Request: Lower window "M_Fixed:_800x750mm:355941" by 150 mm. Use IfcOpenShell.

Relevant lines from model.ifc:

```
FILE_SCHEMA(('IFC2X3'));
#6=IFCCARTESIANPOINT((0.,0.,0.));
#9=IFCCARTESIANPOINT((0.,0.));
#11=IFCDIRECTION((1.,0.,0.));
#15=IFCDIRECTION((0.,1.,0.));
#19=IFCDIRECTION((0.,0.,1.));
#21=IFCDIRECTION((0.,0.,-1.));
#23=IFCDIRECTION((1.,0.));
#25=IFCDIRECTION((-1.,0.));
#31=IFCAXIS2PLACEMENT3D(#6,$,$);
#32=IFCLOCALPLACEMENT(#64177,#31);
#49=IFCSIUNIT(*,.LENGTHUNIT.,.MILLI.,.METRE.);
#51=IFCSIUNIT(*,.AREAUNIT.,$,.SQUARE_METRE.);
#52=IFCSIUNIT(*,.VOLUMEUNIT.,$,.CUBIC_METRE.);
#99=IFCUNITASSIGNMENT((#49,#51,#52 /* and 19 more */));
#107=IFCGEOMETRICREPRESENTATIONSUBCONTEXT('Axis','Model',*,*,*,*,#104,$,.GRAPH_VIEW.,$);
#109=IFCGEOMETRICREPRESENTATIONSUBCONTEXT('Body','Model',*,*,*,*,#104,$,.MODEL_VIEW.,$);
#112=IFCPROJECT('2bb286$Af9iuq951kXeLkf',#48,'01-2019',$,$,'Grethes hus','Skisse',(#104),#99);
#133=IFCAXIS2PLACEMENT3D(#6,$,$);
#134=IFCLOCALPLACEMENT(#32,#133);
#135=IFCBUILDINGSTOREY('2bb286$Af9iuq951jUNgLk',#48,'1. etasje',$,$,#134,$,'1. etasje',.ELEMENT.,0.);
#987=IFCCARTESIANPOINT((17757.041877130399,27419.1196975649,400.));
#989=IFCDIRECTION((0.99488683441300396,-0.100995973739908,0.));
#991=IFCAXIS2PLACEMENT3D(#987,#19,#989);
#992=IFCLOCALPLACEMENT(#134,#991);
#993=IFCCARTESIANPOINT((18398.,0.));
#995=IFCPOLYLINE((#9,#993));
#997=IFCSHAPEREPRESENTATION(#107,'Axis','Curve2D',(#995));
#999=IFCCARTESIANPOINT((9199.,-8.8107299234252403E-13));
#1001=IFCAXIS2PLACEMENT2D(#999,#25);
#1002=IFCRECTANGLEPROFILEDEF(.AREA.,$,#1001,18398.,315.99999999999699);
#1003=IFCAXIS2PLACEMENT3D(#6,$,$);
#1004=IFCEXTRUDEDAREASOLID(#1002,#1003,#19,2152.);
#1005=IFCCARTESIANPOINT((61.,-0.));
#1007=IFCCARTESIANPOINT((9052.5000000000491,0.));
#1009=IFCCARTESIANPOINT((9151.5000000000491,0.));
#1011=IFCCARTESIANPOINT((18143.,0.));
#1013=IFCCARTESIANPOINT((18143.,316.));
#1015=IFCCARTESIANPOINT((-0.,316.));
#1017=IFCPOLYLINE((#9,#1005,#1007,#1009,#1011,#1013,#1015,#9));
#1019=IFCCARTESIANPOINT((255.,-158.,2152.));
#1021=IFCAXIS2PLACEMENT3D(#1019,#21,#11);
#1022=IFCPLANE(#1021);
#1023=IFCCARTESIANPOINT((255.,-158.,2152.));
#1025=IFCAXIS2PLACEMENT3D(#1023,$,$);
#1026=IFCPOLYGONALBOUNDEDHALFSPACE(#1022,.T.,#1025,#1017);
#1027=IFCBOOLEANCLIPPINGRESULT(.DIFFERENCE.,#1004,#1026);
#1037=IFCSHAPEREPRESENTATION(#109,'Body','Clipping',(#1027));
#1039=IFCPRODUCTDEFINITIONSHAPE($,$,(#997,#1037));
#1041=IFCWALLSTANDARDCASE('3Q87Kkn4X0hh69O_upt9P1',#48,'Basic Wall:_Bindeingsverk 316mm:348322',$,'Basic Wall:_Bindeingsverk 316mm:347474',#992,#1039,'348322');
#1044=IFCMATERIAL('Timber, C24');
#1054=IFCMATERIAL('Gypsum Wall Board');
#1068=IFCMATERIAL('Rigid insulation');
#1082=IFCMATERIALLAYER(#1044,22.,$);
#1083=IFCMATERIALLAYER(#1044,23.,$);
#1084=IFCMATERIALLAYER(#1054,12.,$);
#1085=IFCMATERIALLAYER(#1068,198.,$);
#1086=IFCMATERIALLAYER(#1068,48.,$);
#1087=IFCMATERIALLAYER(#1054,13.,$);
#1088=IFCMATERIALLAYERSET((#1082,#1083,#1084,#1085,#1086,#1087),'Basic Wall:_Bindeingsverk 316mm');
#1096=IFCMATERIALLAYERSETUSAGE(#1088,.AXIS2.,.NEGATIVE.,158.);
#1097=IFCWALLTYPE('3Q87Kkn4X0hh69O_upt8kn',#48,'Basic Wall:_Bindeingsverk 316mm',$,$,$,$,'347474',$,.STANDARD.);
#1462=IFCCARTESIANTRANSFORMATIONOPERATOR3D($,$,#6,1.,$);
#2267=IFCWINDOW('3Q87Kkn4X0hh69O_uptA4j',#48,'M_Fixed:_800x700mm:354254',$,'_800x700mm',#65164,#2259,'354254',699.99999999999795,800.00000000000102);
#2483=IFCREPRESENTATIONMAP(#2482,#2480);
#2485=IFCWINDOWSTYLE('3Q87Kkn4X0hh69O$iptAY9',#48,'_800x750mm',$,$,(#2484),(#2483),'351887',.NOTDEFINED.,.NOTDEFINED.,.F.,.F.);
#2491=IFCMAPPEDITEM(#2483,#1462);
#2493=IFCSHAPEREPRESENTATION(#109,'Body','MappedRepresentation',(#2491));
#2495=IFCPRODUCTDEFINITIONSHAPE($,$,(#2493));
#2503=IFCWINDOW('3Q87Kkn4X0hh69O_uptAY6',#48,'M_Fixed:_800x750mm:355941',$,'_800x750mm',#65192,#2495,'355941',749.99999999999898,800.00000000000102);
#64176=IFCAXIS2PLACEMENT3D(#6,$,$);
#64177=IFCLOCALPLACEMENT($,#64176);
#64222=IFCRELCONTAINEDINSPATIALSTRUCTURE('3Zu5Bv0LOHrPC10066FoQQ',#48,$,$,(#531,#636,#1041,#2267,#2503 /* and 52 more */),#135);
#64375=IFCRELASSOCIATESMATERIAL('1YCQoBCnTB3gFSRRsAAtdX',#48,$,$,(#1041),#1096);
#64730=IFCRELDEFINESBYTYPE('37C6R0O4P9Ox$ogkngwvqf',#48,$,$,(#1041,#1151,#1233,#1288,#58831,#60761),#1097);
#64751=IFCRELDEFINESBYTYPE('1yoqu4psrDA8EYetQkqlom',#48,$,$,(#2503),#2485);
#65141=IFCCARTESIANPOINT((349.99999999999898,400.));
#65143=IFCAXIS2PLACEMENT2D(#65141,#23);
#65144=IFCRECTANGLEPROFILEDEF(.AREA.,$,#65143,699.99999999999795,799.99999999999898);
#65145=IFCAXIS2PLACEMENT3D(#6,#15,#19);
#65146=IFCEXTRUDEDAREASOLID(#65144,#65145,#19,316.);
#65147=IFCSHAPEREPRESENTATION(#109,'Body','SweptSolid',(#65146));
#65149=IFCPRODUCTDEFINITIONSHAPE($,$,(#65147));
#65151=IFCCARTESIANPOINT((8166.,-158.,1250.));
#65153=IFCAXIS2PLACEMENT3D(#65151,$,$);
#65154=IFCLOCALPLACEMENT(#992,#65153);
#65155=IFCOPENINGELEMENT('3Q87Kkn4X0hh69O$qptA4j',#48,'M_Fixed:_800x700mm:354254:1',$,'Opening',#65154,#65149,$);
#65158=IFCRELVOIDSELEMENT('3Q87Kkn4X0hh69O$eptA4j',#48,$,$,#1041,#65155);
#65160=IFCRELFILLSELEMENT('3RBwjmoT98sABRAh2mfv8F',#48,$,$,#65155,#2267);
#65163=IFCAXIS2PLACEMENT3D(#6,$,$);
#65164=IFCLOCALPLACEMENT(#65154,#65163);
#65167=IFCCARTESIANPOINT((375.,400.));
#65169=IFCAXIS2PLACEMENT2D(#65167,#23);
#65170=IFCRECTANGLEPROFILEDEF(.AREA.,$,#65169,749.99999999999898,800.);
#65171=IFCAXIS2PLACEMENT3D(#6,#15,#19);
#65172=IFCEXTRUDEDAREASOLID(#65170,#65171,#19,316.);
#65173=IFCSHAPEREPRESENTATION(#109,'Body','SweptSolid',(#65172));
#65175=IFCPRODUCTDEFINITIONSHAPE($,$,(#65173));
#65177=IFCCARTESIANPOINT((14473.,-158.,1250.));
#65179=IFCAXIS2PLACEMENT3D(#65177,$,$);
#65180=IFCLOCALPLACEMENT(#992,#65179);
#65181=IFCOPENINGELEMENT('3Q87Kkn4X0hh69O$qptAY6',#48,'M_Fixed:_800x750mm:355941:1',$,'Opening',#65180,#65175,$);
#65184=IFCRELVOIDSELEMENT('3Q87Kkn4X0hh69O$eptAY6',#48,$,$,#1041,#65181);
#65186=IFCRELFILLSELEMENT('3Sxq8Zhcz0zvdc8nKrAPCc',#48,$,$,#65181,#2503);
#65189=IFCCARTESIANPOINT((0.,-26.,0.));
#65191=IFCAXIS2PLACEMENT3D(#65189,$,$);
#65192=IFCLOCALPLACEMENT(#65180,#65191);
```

```python
import numpy as np
import ifcopenshell
import ifcopenshell.api.geometry
import ifcopenshell.util.placement
import ifcopenshell.util.unit

model = ifcopenshell.open("model.ifc")
unit_scale = ifcopenshell.util.unit.calculate_unit_scale(model)

window = model.by_guid("3Q87Kkn4X0hh69O_uptAY6")
opening = window.FillsVoids[0].RelatingOpeningElement
dz = -150.0

shift = np.array([0.0, 0.0, dz])
# The window is placed relative to its opening, so it follows when the opening moves.
matrix = ifcopenshell.util.placement.get_local_placement(opening.ObjectPlacement)
matrix[:3, 3] += shift
ifcopenshell.api.geometry.edit_object_placement(
    model, product=opening, matrix=matrix, is_si=False, should_transform_children=True
)

print(f"moved by {dz * unit_scale:+.3f} m")

model.write("model_rev.ifc")
```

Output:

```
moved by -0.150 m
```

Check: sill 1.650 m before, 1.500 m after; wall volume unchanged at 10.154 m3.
